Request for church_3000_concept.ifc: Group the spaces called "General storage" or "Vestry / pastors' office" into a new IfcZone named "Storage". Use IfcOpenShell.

First a look at what the model holds.

```python
import ifcopenshell

model = ifcopenshell.open("church_3000_concept.ifc")
print(model.schema)
seen = {}
for space in model.by_type("IfcSpace"):
    seen[space.LongName] = seen.get(space.LongName, 0) + 1
for name, count in sorted(seen.items(), key=str):
    print(count, "x", name)
print("zones:", [z.Name for z in model.by_type("IfcZone")][:20])
```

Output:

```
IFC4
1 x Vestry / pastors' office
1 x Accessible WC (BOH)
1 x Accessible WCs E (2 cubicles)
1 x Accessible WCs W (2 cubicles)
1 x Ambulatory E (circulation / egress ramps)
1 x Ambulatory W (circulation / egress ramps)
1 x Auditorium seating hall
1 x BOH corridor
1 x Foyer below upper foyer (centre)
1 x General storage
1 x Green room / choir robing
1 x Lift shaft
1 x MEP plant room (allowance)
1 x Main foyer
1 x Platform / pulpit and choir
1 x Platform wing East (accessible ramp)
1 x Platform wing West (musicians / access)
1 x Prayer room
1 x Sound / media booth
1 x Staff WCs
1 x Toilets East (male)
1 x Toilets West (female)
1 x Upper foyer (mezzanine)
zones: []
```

```python
import ifcopenshell
import ifcopenshell.api.group
import ifcopenshell.api.root

model = ifcopenshell.open("church_3000_concept.ifc")

names = {"General storage", "Vestry / pastors' office"}
spaces = [s for s in model.by_type("IfcSpace") if s.LongName in names]

zone = ifcopenshell.api.root.create_entity(model, ifc_class="IfcZone", name="Storage")
ifcopenshell.api.group.assign_group(model, products=spaces, group=zone)
print(len(spaces), "spaces in", zone.Name)

model.write("church_3000_concept_updated.ifc")
```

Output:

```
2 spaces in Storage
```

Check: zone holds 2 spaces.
